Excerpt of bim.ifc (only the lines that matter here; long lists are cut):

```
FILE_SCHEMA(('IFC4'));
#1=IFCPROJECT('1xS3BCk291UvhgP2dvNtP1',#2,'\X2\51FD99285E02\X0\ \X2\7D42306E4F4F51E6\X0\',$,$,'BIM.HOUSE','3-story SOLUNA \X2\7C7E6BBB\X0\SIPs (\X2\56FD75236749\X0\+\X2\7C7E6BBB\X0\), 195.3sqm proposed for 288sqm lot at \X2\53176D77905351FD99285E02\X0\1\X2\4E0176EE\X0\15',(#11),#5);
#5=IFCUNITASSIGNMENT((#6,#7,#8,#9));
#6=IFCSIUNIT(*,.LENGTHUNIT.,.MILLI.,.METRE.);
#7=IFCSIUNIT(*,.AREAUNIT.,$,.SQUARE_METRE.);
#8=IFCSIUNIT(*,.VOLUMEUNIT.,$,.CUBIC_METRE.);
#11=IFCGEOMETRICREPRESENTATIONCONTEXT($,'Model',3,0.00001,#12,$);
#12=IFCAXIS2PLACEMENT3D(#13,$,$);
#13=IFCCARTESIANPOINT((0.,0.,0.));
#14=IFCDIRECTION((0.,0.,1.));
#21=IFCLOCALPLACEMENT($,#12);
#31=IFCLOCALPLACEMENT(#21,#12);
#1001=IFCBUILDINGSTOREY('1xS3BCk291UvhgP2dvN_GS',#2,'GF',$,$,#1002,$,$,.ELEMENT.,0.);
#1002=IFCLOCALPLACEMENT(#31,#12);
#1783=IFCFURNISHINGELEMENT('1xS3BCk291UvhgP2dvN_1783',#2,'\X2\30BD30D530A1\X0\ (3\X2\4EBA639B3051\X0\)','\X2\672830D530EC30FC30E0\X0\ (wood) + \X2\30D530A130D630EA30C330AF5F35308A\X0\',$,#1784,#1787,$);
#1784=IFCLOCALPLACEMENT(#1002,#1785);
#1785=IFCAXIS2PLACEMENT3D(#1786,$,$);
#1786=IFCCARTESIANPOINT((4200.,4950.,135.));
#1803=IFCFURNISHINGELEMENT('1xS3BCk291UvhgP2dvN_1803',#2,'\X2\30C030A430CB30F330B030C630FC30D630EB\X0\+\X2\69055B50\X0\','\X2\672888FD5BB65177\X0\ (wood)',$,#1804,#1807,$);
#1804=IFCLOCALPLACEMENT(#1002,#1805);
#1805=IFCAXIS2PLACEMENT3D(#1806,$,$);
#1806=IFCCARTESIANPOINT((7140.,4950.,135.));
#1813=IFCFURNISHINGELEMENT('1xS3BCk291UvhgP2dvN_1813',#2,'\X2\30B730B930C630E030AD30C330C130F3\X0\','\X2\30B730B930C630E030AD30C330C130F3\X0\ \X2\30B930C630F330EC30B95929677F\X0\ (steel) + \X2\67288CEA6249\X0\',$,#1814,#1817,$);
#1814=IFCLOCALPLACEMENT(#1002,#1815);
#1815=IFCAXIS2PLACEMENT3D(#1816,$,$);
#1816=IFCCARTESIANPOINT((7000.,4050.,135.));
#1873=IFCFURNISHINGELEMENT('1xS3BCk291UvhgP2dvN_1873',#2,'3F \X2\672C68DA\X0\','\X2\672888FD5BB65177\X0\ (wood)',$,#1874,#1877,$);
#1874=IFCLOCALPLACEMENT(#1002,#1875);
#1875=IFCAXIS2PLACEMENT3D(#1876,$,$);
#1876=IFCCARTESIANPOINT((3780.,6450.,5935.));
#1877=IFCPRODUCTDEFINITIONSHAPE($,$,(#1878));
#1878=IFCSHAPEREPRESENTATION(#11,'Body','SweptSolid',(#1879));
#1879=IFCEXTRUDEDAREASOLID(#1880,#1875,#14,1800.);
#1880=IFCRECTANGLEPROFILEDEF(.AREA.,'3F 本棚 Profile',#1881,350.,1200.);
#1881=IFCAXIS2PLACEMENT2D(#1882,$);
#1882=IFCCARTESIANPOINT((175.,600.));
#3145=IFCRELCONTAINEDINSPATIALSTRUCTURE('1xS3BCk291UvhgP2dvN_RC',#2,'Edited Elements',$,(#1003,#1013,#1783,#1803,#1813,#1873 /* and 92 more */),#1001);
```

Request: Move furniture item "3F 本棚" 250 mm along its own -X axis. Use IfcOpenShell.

```python
import ifcopenshell
import ifcopenshell.api.geometry
import ifcopenshell.util.placement

model = ifcopenshell.open("bim.ifc")

item = model.by_guid("1xS3BCk291UvhgP2dvN_1873")
matrix = ifcopenshell.util.placement.get_local_placement(item.ObjectPlacement)
matrix[:3, 3] -= matrix[:3, 0] * 250.0
ifcopenshell.api.geometry.edit_object_placement(model, product=item, matrix=matrix, is_si=False)

print(ifcopenshell.util.placement.get_local_placement(item.ObjectPlacement).round(3) + 0.0)

model.write("bim_v2.ifc")
```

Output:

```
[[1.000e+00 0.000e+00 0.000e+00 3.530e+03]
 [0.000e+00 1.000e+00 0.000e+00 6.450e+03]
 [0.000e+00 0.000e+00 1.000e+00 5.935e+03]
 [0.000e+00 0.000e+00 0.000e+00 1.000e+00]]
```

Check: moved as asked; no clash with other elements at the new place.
